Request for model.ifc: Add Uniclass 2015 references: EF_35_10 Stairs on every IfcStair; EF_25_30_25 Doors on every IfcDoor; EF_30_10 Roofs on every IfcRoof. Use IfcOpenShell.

First a look at what the model holds.

```python
import ifcopenshell

model = ifcopenshell.open("model.ifc")
print(model.schema)
print("classifications:", [c.Name for c in model.by_type("IfcClassification")])
for ifc_class in ("IfcDoor", "IfcRoof", "IfcStair", "IfcWall", "IfcWindow"):
    print(ifc_class, len(model.by_type(ifc_class)))
```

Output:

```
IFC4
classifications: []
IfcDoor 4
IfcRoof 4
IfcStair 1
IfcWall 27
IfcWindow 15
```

```python
import ifcopenshell
import ifcopenshell.api.classification

model = ifcopenshell.open("model.ifc")

system = ifcopenshell.api.classification.add_classification(model, classification="Uniclass 2015")

codes = {
    "IfcStair": ("EF_35_10", "Stairs"),
    "IfcDoor": ("EF_25_30_25", "Doors"),
    "IfcRoof": ("EF_30_10", "Roofs"),
}
for ifc_class, (code, name) in codes.items():
    products = model.by_type(ifc_class)
    ifcopenshell.api.classification.add_reference(
        model, products=products, classification=system, identification=code, name=name
    )
    print(code, len(products))

model.write("model_edited.ifc")
```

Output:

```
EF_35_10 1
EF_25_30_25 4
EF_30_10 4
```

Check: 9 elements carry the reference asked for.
